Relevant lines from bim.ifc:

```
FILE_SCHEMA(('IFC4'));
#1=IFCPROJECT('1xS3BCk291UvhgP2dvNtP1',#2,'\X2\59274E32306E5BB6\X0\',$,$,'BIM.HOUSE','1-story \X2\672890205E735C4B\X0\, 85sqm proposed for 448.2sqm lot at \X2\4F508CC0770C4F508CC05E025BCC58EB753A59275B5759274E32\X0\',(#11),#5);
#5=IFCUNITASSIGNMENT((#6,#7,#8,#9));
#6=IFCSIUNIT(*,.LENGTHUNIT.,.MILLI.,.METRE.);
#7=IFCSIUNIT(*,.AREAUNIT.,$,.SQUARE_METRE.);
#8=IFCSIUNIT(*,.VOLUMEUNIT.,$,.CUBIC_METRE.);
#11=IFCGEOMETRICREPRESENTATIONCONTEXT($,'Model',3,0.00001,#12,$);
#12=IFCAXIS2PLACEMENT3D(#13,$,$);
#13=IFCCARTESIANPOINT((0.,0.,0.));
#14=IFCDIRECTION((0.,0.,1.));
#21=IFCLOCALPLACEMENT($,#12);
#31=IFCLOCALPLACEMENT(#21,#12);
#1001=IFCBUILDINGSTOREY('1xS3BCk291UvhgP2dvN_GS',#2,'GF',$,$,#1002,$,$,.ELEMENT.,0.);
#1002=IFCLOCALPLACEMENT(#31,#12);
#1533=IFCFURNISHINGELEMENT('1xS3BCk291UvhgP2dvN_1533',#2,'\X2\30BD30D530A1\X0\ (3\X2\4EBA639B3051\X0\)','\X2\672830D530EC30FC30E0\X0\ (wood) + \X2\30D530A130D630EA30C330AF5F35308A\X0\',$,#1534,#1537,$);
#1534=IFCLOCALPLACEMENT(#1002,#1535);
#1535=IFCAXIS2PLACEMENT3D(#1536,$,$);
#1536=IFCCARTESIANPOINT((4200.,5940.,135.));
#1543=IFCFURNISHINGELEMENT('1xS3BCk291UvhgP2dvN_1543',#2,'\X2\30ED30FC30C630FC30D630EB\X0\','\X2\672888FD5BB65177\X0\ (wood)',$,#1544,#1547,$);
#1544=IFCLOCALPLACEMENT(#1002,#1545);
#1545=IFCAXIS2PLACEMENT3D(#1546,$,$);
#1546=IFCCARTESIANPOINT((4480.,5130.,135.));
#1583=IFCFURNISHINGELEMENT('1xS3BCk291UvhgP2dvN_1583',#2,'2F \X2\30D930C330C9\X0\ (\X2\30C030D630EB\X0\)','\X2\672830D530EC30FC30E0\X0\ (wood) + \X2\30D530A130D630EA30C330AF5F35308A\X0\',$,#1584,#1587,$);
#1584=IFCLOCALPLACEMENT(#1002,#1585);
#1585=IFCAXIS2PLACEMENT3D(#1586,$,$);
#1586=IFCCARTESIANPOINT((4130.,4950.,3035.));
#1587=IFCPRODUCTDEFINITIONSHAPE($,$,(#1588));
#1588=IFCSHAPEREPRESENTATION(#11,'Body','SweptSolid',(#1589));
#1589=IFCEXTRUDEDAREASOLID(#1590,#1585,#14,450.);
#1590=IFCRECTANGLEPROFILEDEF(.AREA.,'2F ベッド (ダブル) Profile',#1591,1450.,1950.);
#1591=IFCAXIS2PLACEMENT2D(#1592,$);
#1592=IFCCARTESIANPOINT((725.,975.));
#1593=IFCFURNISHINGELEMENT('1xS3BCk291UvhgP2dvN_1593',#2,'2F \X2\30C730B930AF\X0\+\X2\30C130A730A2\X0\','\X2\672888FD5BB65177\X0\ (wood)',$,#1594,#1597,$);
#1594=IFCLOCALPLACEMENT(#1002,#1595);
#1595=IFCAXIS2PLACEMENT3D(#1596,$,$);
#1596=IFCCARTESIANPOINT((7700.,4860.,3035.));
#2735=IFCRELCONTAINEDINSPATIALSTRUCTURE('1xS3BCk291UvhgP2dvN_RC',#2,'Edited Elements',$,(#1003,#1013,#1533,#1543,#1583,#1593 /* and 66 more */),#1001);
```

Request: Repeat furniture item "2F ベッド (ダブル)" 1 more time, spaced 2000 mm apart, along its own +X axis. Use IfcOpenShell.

```python
import ifcopenshell
import ifcopenshell.api.geometry
import ifcopenshell.api.root
import ifcopenshell.util.element
import ifcopenshell.util.placement

model = ifcopenshell.open("bim.ifc")


def reuse_history(source, copy):
    """copy_class also copies each property set's owner history, people and application; keep the originals."""
    for rel in copy.IsDefinedBy:
        if rel.is_a("IfcRelDefinesByProperties") and (history := rel.RelatingPropertyDefinition.OwnerHistory):
            rel.RelatingPropertyDefinition.OwnerHistory = source.OwnerHistory
            ifcopenshell.util.element.remove_deep2(model, history)


source = model.by_guid("1xS3BCk291UvhgP2dvN_1583")
base = ifcopenshell.util.placement.get_local_placement(source.ObjectPlacement)
step = base[:3, 0] * 2000.0

for i in range(1, 2):
    copy = ifcopenshell.api.root.copy_class(model, product=source)
    copy.Representation = ifcopenshell.util.element.copy_deep(
        model, source.Representation, exclude=["IfcGeometricRepresentationContext", "IfcRepresentationMap"]
    )
    reuse_history(source, copy)
    matrix = base.copy()
    matrix[:3, 3] += i * step
    print("added at", matrix[:3, 3].round(3) + 0.0)
    ifcopenshell.api.geometry.edit_object_placement(model, product=copy, matrix=matrix, is_si=False)

model.write("bim_updated.ifc")
```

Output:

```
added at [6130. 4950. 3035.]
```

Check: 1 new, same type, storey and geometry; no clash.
